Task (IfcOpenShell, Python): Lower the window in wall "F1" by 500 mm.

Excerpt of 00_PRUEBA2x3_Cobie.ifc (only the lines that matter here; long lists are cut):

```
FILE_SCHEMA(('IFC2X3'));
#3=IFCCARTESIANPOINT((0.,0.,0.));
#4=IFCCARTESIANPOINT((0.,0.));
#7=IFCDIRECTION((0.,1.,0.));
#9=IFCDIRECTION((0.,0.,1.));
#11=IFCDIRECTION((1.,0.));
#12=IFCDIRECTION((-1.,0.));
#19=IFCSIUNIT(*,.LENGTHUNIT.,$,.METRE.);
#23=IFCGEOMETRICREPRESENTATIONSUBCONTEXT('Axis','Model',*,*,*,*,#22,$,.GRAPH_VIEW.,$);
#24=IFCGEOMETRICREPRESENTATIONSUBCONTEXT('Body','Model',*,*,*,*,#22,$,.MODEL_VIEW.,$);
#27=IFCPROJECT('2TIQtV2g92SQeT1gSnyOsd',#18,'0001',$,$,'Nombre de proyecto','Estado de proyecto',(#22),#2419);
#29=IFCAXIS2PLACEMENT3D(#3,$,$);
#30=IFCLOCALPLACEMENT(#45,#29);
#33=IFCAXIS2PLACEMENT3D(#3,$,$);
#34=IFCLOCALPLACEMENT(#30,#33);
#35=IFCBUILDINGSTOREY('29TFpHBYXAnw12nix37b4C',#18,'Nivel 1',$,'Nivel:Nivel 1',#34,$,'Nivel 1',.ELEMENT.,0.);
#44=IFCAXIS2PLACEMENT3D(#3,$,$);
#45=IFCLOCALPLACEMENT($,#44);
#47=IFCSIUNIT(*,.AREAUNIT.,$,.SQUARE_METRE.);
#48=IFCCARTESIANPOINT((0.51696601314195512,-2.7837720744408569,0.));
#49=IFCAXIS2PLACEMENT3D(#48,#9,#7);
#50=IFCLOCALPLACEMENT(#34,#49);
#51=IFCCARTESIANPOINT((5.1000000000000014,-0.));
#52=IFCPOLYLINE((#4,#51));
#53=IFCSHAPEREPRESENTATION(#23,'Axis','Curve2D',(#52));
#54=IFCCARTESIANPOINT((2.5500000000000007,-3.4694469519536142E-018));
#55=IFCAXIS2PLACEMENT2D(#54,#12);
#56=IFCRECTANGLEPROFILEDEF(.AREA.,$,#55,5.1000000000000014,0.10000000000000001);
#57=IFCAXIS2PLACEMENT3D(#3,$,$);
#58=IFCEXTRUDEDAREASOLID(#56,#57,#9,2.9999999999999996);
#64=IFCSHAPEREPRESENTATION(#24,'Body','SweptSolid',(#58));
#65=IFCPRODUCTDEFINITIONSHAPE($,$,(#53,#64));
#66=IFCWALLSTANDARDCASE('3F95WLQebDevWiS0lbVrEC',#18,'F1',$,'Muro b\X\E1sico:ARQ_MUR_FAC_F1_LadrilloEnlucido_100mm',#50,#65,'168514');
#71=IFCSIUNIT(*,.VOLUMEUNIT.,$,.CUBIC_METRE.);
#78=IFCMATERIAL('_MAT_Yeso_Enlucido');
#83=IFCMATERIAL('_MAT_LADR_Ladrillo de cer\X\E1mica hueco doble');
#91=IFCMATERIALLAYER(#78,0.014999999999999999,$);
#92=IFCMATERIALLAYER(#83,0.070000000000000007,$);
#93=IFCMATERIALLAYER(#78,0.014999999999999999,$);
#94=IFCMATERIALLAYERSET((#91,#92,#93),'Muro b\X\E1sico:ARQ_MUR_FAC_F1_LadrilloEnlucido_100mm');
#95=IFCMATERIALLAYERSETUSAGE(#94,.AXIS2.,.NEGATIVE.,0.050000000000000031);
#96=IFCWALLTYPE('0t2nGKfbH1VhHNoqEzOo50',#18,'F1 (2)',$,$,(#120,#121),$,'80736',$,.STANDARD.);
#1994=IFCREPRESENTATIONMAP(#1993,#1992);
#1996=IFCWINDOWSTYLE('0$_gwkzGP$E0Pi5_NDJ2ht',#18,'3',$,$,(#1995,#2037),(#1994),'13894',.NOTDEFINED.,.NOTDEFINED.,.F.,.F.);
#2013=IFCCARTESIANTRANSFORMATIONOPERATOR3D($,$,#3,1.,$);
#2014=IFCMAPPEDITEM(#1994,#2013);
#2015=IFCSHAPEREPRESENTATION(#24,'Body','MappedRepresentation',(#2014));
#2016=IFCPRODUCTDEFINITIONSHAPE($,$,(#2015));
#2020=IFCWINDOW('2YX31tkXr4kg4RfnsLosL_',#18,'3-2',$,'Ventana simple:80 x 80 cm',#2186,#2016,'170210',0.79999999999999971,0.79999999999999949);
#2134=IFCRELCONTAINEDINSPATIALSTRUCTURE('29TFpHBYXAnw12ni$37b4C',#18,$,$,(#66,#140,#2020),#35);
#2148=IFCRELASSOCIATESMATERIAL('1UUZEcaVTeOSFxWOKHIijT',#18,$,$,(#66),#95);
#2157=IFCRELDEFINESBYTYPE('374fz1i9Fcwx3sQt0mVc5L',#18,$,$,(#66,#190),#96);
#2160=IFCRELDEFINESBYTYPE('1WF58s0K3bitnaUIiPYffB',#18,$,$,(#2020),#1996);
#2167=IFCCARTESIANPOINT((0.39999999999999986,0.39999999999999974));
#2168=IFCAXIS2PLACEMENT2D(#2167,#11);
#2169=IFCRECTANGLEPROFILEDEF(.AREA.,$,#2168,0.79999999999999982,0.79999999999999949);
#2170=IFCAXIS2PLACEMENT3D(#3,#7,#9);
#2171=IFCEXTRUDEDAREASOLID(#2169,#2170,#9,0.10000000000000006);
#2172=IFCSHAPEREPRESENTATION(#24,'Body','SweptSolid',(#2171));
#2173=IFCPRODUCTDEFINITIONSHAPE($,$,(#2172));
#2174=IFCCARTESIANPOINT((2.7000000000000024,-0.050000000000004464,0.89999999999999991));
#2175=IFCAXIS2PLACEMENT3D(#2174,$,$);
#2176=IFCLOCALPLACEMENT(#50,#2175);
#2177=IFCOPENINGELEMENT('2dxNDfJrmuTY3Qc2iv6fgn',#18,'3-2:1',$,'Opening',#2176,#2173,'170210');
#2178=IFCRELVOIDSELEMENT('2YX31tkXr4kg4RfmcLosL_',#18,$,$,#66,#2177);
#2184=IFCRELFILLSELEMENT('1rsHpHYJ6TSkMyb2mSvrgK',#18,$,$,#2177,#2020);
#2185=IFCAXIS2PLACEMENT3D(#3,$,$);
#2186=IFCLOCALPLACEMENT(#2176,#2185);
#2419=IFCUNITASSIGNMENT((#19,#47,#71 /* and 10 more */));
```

```python
import numpy as np
import ifcopenshell
import ifcopenshell.api.geometry
import ifcopenshell.util.placement
import ifcopenshell.util.unit

model = ifcopenshell.open("00_PRUEBA2x3_Cobie.ifc")
unit_scale = ifcopenshell.util.unit.calculate_unit_scale(model)

window = model.by_guid("2YX31tkXr4kg4RfnsLosL_")
opening = window.FillsVoids[0].RelatingOpeningElement
dz = -0.5 / unit_scale

shift = np.array([0.0, 0.0, dz])
# The window is placed relative to its opening, so it follows when the opening moves.
matrix = ifcopenshell.util.placement.get_local_placement(opening.ObjectPlacement)
matrix[:3, 3] += shift
ifcopenshell.api.geometry.edit_object_placement(
    model, product=opening, matrix=matrix, is_si=False, should_transform_children=True
)

print(f"moved by {dz * unit_scale:+.3f} m")

model.write("00_PRUEBA2x3_Cobie_updated.ifc")
```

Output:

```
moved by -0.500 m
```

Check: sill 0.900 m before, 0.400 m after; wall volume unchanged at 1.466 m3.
